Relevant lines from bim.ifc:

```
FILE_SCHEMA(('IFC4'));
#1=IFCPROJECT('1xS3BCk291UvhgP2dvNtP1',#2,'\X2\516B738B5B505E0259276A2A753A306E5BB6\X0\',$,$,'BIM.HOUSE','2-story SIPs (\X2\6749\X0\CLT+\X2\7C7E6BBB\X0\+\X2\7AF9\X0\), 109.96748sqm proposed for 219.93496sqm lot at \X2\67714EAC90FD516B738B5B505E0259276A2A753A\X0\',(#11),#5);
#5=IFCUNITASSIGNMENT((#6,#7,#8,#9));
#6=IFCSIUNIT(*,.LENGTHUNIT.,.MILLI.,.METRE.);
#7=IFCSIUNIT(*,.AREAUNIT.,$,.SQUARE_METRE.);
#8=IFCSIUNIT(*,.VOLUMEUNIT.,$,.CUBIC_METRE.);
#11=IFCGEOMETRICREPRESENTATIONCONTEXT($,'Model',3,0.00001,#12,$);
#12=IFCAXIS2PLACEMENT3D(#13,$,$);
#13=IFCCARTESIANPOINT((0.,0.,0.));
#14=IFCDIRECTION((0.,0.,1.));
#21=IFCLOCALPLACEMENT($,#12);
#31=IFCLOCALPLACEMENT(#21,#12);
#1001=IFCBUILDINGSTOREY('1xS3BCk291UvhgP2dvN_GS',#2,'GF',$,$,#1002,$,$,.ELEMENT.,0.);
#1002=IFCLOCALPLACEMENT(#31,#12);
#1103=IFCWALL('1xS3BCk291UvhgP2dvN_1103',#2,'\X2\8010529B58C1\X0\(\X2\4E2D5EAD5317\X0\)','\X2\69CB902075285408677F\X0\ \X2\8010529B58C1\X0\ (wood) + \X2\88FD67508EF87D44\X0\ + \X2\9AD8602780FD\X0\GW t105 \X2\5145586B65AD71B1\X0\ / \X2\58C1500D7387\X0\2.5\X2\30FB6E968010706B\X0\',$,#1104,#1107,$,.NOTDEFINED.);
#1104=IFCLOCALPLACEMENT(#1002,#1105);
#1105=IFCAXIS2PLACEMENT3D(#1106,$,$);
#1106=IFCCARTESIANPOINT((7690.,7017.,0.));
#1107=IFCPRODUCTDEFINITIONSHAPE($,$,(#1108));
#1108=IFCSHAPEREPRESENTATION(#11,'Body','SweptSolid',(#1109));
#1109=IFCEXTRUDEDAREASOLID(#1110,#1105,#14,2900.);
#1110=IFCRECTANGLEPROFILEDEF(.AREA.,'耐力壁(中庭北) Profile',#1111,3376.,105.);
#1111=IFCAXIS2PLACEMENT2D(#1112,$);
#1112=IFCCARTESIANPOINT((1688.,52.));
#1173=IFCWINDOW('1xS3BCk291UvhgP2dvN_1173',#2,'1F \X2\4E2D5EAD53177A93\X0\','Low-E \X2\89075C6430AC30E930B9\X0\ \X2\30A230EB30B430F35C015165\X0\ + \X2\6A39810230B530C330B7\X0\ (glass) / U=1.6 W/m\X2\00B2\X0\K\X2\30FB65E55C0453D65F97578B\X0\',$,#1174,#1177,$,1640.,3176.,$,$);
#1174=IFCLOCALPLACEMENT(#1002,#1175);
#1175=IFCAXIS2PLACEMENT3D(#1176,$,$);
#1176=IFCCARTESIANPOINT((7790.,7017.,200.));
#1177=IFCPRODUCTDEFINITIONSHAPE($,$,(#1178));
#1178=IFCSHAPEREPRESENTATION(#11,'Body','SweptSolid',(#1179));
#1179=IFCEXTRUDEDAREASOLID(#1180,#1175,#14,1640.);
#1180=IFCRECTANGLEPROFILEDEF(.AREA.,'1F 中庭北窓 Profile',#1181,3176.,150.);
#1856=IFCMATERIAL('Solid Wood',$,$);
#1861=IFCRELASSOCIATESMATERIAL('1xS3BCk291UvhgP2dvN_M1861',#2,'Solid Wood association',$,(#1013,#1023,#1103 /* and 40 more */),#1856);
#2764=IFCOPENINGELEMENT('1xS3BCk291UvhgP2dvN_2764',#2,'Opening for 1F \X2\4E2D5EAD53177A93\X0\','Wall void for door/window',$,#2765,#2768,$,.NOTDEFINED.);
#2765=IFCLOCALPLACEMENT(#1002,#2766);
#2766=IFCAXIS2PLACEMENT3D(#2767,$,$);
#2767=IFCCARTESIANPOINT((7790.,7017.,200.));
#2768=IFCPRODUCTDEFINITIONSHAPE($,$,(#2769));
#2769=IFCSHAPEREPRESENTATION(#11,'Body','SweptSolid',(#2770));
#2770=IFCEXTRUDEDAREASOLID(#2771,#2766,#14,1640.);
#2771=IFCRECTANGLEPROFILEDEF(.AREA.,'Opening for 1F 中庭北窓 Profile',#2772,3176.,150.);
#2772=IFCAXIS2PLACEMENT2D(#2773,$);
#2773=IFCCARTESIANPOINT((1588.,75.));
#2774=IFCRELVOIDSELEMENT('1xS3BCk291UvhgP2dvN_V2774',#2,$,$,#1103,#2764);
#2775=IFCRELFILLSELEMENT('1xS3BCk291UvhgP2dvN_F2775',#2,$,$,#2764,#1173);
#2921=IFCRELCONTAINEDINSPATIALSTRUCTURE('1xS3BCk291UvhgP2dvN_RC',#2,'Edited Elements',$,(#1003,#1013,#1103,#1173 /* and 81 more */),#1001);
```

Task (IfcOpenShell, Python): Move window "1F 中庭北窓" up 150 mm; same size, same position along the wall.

```python
import numpy as np
import ifcopenshell
import ifcopenshell.api.geometry
import ifcopenshell.util.placement
import ifcopenshell.util.unit

model = ifcopenshell.open("bim.ifc")
unit_scale = ifcopenshell.util.unit.calculate_unit_scale(model)

window = model.by_guid("1xS3BCk291UvhgP2dvN_1173")
opening = window.FillsVoids[0].RelatingOpeningElement
dz = 0.15 / unit_scale

shift = np.array([0.0, 0.0, dz])
# The window is not placed relative to its opening, so move both.
for product in (opening, window):
    matrix = ifcopenshell.util.placement.get_local_placement(product.ObjectPlacement)
    matrix[:3, 3] += shift
    ifcopenshell.api.geometry.edit_object_placement(model, product=product, matrix=matrix, is_si=False)

print(f"moved by {dz * unit_scale:+.3f} m")

model.write("bim_v2.ifc")
```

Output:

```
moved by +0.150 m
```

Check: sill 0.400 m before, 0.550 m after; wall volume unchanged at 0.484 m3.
